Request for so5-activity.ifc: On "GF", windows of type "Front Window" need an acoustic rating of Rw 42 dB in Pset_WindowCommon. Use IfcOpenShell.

First a look at what the model holds.

```python
import ifcopenshell
import ifcopenshell.util.element

model = ifcopenshell.open("so5-activity.ifc")
print(model.schema)
storey = next(s for s in model.by_type("IfcBuildingStorey") if s.Name == "GF")
windows = [e for e in ifcopenshell.util.element.get_decomposition(storey) if e.is_a("IfcWindow")]
seen = {}
for e in windows:
    element_type = ifcopenshell.util.element.get_type(e)
    key = (element_type.Name if element_type != e and element_type else None, ifcopenshell.util.element.get_pset(e, "Pset_WindowCommon", "AcousticRating"))
    seen[key] = seen.get(key, 0) + 1
for (name, value), count in sorted(seen.items(), key=str):
    print(count, "x", name, "|", value)
```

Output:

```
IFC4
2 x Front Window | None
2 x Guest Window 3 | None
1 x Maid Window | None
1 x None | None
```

```python
import ifcopenshell
import ifcopenshell.api.pset
import ifcopenshell.util.element

model = ifcopenshell.open("so5-activity.ifc")

storey = next(s for s in model.by_type("IfcBuildingStorey") if s.Name == "GF")
windows = [e for e in ifcopenshell.util.element.get_decomposition(storey) if e.is_a("IfcWindow")]

count = 0
for e in windows:
    element_type = ifcopenshell.util.element.get_type(e)
    if element_type in (None, e) or element_type.Name != "Front Window":
        continue
    # add_pset returns the element's existing set when there is one.
    pset = ifcopenshell.api.pset.add_pset(model, product=e, name="Pset_WindowCommon")
    ifcopenshell.api.pset.edit_pset(model, pset=pset, properties={"AcousticRating": "Rw 42 dB"})
    count += 1

print(count, "windows updated")

model.write("so5-activity-out.ifc")
```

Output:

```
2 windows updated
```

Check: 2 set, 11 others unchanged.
